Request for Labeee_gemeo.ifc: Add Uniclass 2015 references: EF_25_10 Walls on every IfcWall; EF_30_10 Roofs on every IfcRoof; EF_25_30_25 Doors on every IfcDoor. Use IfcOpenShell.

First a look at what the model holds.

```python
import ifcopenshell

model = ifcopenshell.open("Labeee_gemeo.ifc")
print(model.schema)
print("classifications:", [c.Name for c in model.by_type("IfcClassification")])
for ifc_class in ("IfcDoor", "IfcRoof", "IfcStair", "IfcWall", "IfcWindow"):
    print(ifc_class, len(model.by_type(ifc_class)))
```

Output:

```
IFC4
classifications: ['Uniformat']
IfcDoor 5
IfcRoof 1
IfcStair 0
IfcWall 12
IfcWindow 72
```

```python
import ifcopenshell
import ifcopenshell.api.classification

model = ifcopenshell.open("Labeee_gemeo.ifc")

system = ifcopenshell.api.classification.add_classification(model, classification="Uniclass 2015")

codes = {
    "IfcWall": ("EF_25_10", "Walls"),
    "IfcRoof": ("EF_30_10", "Roofs"),
    "IfcDoor": ("EF_25_30_25", "Doors"),
}
for ifc_class, (code, name) in codes.items():
    products = model.by_type(ifc_class)
    ifcopenshell.api.classification.add_reference(
        model, products=products, classification=system, identification=code, name=name
    )
    print(code, len(products))

model.write("Labeee_gemeo_updated.ifc")
```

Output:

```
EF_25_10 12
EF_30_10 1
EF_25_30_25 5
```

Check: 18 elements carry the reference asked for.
